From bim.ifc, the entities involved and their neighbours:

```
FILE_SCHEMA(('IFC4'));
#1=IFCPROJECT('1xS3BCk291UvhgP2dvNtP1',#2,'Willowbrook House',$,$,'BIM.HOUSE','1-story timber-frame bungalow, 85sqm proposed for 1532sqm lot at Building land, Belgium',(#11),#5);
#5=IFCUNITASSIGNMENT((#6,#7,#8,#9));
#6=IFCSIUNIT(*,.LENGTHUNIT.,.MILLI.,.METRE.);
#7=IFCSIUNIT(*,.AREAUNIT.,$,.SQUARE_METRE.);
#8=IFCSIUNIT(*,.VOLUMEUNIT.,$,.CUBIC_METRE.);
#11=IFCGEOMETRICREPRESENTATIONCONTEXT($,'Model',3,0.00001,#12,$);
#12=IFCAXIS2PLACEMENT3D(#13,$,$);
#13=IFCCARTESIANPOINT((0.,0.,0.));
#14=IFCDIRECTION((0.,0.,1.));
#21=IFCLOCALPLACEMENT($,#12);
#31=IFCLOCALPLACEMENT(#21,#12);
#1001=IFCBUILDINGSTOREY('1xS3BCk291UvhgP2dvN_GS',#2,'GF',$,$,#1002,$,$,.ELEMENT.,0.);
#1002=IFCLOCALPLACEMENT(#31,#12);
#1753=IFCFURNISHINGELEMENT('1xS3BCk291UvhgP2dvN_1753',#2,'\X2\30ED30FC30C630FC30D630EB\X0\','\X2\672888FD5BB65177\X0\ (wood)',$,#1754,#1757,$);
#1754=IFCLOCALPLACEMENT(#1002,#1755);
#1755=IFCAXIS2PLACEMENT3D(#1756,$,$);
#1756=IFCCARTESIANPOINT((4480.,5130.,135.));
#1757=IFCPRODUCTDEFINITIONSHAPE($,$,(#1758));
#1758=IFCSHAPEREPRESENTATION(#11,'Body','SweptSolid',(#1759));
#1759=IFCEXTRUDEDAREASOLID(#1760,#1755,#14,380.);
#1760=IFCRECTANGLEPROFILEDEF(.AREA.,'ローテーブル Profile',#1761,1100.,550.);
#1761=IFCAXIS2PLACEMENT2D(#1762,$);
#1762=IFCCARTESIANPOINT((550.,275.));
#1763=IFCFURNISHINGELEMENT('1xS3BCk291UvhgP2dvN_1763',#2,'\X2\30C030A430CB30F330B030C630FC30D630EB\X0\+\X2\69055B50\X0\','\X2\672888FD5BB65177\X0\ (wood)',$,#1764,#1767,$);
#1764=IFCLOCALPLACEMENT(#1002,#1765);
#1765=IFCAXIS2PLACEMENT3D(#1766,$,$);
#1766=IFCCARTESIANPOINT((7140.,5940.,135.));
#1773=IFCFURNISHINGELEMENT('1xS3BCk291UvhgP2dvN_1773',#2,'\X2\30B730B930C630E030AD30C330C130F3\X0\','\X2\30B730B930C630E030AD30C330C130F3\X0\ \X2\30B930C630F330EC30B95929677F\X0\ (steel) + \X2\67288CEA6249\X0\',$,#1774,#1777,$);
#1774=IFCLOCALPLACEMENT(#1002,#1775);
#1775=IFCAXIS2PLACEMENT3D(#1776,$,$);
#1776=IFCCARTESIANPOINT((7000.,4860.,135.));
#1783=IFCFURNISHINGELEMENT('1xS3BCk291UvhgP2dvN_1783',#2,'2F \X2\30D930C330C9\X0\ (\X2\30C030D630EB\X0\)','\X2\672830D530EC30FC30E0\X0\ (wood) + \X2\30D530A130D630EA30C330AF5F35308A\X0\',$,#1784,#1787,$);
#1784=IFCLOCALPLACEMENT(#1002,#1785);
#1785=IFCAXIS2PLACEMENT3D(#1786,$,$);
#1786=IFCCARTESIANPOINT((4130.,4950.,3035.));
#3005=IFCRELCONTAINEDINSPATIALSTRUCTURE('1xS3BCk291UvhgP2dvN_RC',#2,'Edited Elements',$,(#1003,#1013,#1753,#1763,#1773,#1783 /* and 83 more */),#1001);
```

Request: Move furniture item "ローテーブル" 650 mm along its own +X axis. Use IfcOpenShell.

```python
import ifcopenshell
import ifcopenshell.api.geometry
import ifcopenshell.util.placement

model = ifcopenshell.open("bim.ifc")

item = model.by_id(1753)
matrix = ifcopenshell.util.placement.get_local_placement(item.ObjectPlacement)
matrix[:3, 3] += matrix[:3, 0] * 650.0
ifcopenshell.api.geometry.edit_object_placement(model, product=item, matrix=matrix, is_si=False)

print(ifcopenshell.util.placement.get_local_placement(item.ObjectPlacement).round(3) + 0.0)

model.write("bim_edited.ifc")
```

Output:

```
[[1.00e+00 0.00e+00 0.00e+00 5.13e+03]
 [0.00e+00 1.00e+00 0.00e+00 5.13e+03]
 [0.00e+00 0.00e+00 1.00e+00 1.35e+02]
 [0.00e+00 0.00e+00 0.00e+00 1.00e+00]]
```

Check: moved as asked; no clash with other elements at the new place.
